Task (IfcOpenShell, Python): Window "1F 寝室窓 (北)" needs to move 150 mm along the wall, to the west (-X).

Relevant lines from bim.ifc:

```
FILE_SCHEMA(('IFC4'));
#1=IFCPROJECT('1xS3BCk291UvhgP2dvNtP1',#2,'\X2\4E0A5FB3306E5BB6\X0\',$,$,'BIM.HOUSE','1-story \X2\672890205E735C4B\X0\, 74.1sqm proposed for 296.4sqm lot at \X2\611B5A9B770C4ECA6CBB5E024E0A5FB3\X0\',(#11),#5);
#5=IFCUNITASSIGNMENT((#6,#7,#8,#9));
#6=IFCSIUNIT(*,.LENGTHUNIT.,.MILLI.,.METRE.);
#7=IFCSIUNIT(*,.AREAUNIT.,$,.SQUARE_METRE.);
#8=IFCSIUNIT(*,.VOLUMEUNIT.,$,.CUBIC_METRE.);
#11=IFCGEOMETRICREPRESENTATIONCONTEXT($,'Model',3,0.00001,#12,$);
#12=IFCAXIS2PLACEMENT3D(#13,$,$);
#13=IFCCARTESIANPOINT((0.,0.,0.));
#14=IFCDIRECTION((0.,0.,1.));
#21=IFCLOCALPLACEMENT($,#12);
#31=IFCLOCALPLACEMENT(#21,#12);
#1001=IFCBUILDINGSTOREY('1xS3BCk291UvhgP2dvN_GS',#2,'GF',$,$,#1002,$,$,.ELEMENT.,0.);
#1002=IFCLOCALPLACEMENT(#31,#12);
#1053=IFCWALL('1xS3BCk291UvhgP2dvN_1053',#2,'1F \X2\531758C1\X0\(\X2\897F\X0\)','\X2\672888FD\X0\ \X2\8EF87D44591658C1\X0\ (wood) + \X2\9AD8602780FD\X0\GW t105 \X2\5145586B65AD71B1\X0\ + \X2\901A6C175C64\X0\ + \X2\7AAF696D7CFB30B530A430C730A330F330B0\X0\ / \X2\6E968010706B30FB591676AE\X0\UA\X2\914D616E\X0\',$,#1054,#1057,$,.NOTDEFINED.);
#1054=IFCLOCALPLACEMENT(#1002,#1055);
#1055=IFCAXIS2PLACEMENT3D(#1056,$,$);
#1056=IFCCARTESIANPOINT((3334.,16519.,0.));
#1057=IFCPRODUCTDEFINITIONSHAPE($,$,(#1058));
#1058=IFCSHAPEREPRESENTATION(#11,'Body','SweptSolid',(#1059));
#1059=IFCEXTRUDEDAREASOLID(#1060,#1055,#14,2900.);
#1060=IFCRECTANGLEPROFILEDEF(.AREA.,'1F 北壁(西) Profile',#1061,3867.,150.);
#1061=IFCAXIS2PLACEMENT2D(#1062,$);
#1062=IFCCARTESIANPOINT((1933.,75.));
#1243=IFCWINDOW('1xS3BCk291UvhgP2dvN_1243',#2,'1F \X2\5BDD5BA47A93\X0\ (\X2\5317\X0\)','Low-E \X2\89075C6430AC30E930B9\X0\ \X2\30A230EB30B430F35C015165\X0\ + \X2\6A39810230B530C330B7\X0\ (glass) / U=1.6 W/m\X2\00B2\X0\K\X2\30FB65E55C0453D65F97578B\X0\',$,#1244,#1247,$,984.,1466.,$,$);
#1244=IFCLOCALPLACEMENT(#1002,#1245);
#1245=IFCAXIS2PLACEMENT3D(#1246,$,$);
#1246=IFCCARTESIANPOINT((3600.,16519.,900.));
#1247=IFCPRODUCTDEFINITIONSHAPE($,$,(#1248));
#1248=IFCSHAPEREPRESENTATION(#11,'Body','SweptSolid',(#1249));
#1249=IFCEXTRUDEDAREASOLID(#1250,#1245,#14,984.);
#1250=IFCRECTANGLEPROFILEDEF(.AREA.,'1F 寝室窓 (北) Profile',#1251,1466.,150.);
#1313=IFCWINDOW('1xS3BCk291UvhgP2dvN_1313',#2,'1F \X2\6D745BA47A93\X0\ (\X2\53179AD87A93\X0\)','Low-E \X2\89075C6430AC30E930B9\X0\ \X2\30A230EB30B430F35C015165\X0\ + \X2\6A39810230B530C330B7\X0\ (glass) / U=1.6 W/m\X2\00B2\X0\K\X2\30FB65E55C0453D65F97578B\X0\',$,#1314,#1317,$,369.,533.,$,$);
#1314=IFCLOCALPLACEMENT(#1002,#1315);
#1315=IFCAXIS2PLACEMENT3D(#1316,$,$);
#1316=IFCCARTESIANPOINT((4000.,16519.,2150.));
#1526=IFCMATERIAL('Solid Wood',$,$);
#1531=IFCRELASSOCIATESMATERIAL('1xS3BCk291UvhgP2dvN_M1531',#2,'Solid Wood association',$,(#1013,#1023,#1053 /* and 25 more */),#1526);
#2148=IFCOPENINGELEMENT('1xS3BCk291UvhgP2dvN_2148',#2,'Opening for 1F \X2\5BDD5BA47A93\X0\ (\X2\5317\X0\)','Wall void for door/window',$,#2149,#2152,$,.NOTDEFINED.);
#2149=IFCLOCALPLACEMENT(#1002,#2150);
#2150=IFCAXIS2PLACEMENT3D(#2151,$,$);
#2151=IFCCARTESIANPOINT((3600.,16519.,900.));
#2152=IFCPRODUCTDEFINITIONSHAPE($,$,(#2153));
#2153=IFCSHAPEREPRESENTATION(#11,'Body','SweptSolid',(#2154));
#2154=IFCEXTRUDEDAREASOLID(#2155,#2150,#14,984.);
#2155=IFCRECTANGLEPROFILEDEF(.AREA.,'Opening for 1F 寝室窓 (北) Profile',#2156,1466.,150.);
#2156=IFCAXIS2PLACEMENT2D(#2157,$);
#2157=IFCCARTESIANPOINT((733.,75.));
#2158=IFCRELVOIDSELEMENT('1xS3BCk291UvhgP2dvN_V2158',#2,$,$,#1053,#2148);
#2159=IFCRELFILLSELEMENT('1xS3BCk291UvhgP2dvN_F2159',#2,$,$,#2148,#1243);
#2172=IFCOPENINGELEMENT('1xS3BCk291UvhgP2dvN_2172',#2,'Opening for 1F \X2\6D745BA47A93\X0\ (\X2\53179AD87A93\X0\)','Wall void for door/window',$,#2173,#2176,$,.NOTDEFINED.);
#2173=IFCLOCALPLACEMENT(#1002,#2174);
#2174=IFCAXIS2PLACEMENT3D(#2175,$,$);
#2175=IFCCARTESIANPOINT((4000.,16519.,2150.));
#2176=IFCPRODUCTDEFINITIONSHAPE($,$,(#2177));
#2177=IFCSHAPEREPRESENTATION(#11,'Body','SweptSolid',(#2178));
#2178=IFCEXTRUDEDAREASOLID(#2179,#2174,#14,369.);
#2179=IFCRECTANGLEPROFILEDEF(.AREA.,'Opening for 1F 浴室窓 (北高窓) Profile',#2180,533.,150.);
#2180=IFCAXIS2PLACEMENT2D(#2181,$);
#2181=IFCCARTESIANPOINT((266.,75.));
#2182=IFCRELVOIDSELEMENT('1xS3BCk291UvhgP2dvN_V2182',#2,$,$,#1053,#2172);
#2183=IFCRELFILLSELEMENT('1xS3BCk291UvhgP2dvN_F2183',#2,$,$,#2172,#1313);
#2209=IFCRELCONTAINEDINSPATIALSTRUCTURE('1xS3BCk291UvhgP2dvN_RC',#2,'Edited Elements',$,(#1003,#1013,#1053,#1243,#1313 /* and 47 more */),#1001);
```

```python
import ifcopenshell
import ifcopenshell.api.geometry
import ifcopenshell.util.placement
import ifcopenshell.util.unit

model = ifcopenshell.open("bim.ifc")
unit_scale = ifcopenshell.util.unit.calculate_unit_scale(model)

window = model.by_id(1243)
opening = window.FillsVoids[0].RelatingOpeningElement
wall = opening.VoidsElements[0].RelatingBuildingElement

wall_matrix = ifcopenshell.util.placement.get_local_placement(wall.ObjectPlacement)
shift = wall_matrix[:3, 0] * -0.15 / unit_scale
before = ifcopenshell.util.placement.get_local_placement(window.ObjectPlacement)[:3, 3].copy()

# The window is not placed relative to its opening, so move both.
for product in (opening, window):
    matrix = ifcopenshell.util.placement.get_local_placement(product.ObjectPlacement)
    matrix[:3, 3] += shift
    ifcopenshell.api.geometry.edit_object_placement(model, product=product, matrix=matrix, is_si=False)

after = ifcopenshell.util.placement.get_local_placement(window.ObjectPlacement)[:3, 3]
print("window moved by", (after - before).round(3) + 0.0)

model.write("bim_rev.ifc")
```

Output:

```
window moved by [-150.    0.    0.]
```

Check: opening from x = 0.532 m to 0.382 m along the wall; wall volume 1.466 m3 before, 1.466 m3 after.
